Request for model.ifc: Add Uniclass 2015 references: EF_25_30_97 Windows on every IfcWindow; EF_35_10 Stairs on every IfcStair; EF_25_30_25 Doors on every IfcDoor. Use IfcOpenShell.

First a look at what the model holds.

```python
import ifcopenshell

model = ifcopenshell.open("model.ifc")
print(model.schema)
print("classifications:", [c.Name for c in model.by_type("IfcClassification")])
for ifc_class in ("IfcDoor", "IfcRoof", "IfcStair", "IfcWall", "IfcWindow"):
    print(ifc_class, len(model.by_type(ifc_class)))
```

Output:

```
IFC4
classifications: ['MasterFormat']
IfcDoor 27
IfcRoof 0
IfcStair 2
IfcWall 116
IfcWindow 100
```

```python
import ifcopenshell
import ifcopenshell.api.classification

model = ifcopenshell.open("model.ifc")

system = ifcopenshell.api.classification.add_classification(model, classification="Uniclass 2015")

codes = {
    "IfcWindow": ("EF_25_30_97", "Windows"),
    "IfcStair": ("EF_35_10", "Stairs"),
    "IfcDoor": ("EF_25_30_25", "Doors"),
}
for ifc_class, (code, name) in codes.items():
    products = model.by_type(ifc_class)
    ifcopenshell.api.classification.add_reference(
        model, products=products, classification=system, identification=code, name=name
    )
    print(code, len(products))

model.write("model_rev.ifc")
```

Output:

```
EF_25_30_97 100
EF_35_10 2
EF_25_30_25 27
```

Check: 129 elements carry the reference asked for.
